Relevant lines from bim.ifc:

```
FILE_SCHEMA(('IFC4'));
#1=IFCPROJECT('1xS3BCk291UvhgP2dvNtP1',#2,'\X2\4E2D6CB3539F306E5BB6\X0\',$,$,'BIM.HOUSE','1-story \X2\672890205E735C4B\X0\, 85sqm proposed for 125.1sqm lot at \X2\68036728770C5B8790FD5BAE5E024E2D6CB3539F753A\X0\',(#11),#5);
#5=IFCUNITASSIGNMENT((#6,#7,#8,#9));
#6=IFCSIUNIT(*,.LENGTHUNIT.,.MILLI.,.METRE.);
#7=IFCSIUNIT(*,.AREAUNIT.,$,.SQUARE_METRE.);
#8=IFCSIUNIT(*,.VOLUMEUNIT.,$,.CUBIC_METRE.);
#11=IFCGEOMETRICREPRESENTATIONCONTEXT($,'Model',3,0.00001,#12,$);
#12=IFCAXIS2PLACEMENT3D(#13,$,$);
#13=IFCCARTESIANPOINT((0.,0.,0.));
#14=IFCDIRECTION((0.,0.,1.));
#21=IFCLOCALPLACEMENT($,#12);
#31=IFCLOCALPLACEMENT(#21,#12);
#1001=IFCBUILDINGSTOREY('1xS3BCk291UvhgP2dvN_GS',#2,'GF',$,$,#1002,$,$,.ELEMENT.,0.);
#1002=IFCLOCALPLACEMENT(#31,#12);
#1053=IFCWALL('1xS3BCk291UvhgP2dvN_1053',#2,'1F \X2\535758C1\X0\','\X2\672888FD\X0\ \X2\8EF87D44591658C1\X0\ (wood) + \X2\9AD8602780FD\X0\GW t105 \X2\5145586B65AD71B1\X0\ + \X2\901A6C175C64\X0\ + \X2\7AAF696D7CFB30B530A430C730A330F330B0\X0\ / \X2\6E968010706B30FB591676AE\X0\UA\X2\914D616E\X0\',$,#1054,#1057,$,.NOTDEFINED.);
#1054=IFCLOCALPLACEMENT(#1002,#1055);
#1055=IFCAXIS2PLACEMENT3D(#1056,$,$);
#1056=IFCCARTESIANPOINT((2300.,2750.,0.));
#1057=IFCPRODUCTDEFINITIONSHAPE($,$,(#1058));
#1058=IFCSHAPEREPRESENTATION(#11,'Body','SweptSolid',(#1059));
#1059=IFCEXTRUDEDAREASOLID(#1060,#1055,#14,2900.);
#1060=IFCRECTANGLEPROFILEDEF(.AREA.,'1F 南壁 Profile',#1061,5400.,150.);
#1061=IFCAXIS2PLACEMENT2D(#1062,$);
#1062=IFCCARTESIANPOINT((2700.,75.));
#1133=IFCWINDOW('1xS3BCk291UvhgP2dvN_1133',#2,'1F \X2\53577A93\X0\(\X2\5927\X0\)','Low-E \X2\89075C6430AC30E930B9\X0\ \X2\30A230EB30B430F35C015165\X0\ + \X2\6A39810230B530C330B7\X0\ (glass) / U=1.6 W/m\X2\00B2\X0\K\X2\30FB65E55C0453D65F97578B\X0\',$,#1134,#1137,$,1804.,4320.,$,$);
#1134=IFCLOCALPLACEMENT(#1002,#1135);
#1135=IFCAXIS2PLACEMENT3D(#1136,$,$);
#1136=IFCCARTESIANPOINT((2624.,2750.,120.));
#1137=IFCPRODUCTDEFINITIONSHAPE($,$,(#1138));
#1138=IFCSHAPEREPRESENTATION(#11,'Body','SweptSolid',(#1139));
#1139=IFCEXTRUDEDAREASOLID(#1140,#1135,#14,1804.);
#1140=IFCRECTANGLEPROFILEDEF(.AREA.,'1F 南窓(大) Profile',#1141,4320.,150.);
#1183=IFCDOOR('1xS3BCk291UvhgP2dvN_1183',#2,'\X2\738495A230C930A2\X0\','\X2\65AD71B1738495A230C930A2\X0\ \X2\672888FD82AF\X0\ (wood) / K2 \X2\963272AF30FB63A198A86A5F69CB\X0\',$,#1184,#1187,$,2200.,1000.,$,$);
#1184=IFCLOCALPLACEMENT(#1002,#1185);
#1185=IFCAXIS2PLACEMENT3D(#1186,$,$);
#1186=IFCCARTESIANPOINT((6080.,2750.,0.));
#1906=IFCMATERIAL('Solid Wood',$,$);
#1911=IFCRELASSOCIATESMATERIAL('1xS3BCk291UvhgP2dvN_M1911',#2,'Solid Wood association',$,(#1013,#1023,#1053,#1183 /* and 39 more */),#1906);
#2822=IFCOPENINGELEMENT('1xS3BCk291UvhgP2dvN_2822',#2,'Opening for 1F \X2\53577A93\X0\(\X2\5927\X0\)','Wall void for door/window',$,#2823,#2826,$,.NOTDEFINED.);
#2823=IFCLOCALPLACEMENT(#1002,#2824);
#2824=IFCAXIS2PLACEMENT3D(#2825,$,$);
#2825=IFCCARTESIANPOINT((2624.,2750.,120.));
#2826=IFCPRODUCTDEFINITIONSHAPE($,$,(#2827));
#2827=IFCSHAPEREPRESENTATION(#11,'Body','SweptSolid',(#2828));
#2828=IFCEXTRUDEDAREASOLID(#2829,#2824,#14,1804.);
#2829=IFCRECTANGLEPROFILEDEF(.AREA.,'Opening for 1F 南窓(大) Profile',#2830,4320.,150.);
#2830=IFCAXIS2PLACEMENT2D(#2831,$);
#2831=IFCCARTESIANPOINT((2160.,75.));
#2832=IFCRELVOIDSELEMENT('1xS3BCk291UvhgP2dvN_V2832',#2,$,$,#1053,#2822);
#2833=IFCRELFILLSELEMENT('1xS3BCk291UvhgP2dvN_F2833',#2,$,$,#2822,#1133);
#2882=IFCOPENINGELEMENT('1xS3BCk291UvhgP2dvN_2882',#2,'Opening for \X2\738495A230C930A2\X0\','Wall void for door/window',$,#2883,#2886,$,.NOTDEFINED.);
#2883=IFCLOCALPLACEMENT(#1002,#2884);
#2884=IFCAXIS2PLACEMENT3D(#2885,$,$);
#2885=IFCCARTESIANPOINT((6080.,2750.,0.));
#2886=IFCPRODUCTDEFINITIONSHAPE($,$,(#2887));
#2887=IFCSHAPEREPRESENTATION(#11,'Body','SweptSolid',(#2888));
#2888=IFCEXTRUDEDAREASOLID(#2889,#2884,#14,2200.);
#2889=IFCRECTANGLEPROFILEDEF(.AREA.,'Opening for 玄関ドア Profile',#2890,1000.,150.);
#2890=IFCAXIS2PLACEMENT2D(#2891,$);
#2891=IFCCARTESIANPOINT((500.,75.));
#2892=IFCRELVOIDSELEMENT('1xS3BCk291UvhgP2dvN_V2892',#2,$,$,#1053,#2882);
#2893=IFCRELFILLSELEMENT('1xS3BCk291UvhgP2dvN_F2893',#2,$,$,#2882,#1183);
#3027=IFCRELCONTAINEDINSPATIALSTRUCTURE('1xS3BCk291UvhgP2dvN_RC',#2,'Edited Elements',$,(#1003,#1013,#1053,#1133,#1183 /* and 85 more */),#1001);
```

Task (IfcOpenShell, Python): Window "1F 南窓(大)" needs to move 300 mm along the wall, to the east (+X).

```python
import ifcopenshell
import ifcopenshell.api.geometry
import ifcopenshell.util.placement

model = ifcopenshell.open("bim.ifc")

window = model.by_id(1133)
opening = window.FillsVoids[0].RelatingOpeningElement
wall = opening.VoidsElements[0].RelatingBuildingElement

wall_matrix = ifcopenshell.util.placement.get_local_placement(wall.ObjectPlacement)
shift = wall_matrix[:3, 0] * 300.0
before = ifcopenshell.util.placement.get_local_placement(window.ObjectPlacement)[:3, 3].copy()

# The window is not placed relative to its opening, so move both.
for product in (opening, window):
    matrix = ifcopenshell.util.placement.get_local_placement(product.ObjectPlacement)
    matrix[:3, 3] += shift
    ifcopenshell.api.geometry.edit_object_placement(model, product=product, matrix=matrix, is_si=False)

after = ifcopenshell.util.placement.get_local_placement(window.ObjectPlacement)[:3, 3]
print("window moved by", (after - before).round(3) + 0.0)

model.write("bim_edited.ifc")
```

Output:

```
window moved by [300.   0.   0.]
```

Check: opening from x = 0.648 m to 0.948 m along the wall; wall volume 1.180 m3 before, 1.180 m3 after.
